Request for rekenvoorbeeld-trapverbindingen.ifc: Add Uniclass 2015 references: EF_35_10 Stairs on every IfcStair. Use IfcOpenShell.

First a look at what the model holds.

```python
import ifcopenshell

model = ifcopenshell.open("rekenvoorbeeld-trapverbindingen.ifc")
print(model.schema)
print("classifications:", [c.Name for c in model.by_type("IfcClassification")])
for ifc_class in ("IfcDoor", "IfcRoof", "IfcStair", "IfcWall", "IfcWindow"):
    print(ifc_class, len(model.by_type(ifc_class)))
```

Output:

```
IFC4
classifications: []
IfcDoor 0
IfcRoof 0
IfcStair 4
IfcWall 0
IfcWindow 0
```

```python
import ifcopenshell
import ifcopenshell.api.classification

model = ifcopenshell.open("rekenvoorbeeld-trapverbindingen.ifc")

system = ifcopenshell.api.classification.add_classification(model, classification="Uniclass 2015")

codes = {
    "IfcStair": ("EF_35_10", "Stairs"),
}
for ifc_class, (code, name) in codes.items():
    products = model.by_type(ifc_class)
    ifcopenshell.api.classification.add_reference(
        model, products=products, classification=system, identification=code, name=name
    )
    print(code, len(products))

model.write("rekenvoorbeeld-trapverbindingen_v2.ifc")
```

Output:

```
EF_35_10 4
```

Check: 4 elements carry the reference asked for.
